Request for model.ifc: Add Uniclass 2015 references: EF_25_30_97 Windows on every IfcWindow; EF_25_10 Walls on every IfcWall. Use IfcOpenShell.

First a look at what the model holds.

```python
import ifcopenshell

model = ifcopenshell.open("model.ifc")
print(model.schema)
print("classifications:", [c.Name for c in model.by_type("IfcClassification")])
for ifc_class in ("IfcDoor", "IfcRoof", "IfcStair", "IfcWall", "IfcWindow"):
    print(ifc_class, len(model.by_type(ifc_class)))
```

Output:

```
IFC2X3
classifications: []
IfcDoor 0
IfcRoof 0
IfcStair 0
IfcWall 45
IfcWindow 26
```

```python
import ifcopenshell
import ifcopenshell.api.classification

model = ifcopenshell.open("model.ifc")

# IFC2X3 requires Source and Edition and has no link from the project to the system.
system = model.create_entity("IfcClassification", Source="NBS", Edition="2015", Name="Uniclass 2015")

codes = {
    "IfcWindow": ("EF_25_30_97", "Windows"),
    "IfcWall": ("EF_25_10", "Walls"),
}
for ifc_class, (code, name) in codes.items():
    products = model.by_type(ifc_class)
    ifcopenshell.api.classification.add_reference(
        model, products=products, classification=system, identification=code, name=name
    )
    print(code, len(products))

model.write("model_updated.ifc")
```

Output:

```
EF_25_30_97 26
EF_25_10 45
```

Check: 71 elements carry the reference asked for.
